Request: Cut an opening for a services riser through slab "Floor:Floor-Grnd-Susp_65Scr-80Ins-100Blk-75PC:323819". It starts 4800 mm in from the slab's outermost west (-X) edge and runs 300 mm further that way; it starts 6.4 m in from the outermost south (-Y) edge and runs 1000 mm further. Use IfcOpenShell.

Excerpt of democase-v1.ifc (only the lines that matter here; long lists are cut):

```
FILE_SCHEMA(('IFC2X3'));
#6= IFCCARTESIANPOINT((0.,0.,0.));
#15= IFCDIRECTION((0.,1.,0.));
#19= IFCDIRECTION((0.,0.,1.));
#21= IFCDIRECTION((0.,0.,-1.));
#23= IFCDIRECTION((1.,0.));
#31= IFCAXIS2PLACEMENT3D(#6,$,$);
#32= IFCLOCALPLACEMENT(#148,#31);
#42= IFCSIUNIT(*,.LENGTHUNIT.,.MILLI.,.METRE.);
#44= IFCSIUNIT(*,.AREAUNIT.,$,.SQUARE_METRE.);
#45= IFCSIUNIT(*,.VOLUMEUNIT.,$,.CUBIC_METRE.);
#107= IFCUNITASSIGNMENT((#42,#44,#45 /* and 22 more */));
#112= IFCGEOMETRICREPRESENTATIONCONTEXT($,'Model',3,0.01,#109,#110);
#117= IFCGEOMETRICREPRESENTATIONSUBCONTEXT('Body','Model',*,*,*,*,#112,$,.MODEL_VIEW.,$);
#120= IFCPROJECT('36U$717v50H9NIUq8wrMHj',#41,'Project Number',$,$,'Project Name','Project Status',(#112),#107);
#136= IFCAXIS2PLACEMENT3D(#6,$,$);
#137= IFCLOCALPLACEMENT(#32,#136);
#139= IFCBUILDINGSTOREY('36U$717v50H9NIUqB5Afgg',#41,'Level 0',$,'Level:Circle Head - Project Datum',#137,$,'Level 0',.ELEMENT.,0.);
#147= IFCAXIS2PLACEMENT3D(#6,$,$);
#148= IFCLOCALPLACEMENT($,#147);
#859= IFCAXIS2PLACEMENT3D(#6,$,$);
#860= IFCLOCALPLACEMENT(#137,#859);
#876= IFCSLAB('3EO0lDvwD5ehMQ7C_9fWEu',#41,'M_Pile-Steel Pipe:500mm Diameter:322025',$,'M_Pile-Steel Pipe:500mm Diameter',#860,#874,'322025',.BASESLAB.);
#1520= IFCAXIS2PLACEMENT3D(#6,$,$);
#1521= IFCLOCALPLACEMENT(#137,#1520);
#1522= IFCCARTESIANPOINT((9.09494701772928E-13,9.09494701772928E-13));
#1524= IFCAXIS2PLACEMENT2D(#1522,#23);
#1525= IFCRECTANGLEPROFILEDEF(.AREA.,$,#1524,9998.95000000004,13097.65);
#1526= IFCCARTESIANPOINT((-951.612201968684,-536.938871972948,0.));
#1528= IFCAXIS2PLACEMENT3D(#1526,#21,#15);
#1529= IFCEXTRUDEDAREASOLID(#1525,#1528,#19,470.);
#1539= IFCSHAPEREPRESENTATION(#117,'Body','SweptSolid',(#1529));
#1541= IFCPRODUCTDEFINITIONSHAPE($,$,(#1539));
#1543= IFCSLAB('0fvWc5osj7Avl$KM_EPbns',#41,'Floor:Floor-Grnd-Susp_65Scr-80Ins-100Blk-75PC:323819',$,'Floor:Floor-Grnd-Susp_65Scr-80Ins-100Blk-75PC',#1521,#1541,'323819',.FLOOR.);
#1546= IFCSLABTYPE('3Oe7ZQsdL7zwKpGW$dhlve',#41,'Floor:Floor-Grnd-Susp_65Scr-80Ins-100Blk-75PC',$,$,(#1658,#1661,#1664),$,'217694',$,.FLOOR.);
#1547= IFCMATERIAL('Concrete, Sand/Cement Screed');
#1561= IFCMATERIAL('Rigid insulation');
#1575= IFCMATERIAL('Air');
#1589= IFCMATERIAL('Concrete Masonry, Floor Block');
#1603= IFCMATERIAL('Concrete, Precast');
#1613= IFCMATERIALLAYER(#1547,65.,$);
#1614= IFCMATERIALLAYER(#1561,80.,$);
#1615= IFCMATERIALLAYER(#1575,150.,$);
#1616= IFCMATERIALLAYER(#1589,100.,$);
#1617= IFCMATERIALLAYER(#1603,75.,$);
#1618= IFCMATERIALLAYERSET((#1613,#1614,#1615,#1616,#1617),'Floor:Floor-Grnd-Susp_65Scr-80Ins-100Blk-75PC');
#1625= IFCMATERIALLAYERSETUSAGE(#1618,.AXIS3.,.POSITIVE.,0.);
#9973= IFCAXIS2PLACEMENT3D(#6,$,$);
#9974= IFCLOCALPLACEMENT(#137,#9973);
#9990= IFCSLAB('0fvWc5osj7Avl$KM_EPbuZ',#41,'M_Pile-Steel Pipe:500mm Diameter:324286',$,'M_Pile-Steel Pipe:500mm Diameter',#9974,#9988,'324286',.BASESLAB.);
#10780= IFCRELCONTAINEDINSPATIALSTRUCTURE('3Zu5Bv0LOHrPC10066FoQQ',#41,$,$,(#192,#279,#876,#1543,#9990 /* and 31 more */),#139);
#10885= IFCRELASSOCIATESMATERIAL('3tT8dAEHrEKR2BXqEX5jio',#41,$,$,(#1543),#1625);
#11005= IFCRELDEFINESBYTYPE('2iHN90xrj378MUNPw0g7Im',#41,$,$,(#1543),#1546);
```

```python
import numpy as np
import ifcopenshell
import ifcopenshell.api.feature
import ifcopenshell.api.geometry
import ifcopenshell.api.root
import ifcopenshell.geom
import ifcopenshell.util.placement
import ifcopenshell.util.representation
import ifcopenshell.util.shape
import ifcopenshell.util.unit

model = ifcopenshell.open("democase-v1.ifc")
unit_scale = ifcopenshell.util.unit.calculate_unit_scale(model)
settings = ifcopenshell.geom.settings()


def volume(element):
    """Net volume in cubic metres, openings subtracted."""
    shape = ifcopenshell.geom.create_shape(settings, element)
    return ifcopenshell.util.shape.get_volume(shape.geometry)


slab = model.by_guid("0fvWc5osj7Avl$KM_EPbns")
before = volume(slab)

# Extent in the slab's own axes, in metres. The edges named are its -X and -Y sides.
slab_shape = ifcopenshell.geom.create_shape(settings, slab)
vertices = ifcopenshell.util.shape.get_vertices(slab_shape.geometry)
x_min, y_min, bottom = vertices.min(axis=0)
top = vertices[:, 2].max()

opening = ifcopenshell.api.root.create_entity(model, ifc_class="IfcOpeningElement", name="Services riser opening")
context = ifcopenshell.util.representation.get_context(model, "Model", "Body", "MODEL_VIEW")
width, depth = 0.3, 1
outline = [(0.0, 0.0), (width, 0.0), (width, depth), (0.0, depth), (0.0, 0.0)]
# Overshoot both faces by 50 mm so the cut is clean.
shape = ifcopenshell.api.geometry.add_slab_representation(
    model, context=context, depth=top - bottom + 0.1, polyline=outline
)
ifcopenshell.api.geometry.assign_representation(model, product=opening, representation=shape)

matrix = ifcopenshell.util.placement.get_local_placement(slab.ObjectPlacement)
matrix[:, 3] = matrix @ np.append(np.array([x_min + 4.8, y_min + 6.4, bottom - 0.05]) / unit_scale, 1.0)
ifcopenshell.api.geometry.edit_object_placement(model, product=opening, matrix=matrix, is_si=False)
ifcopenshell.api.feature.add_feature(model, feature=opening, element=slab)

after = volume(slab)

print(f"slab volume {before:.3f} -> {after:.3f} m3")

model.write("democase-v1_rev.ifc")
```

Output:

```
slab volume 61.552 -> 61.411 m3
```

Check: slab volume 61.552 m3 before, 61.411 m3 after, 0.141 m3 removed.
